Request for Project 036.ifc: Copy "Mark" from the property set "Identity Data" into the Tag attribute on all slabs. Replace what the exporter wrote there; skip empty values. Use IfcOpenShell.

First a look at what the model holds.

```python
import ifcopenshell
import ifcopenshell.util.element

model = ifcopenshell.open("Project 036.ifc")
print(model.schema)
slabs = model.by_type("IfcSlab")
print(len(slabs), "slabs")
for e in slabs[:8]:
    source = ifcopenshell.util.element.get_pset(e, "Identity Data", "Mark")
    target = e.Tag
    print(e.id(), repr(source), repr(target), sep=" | ")
```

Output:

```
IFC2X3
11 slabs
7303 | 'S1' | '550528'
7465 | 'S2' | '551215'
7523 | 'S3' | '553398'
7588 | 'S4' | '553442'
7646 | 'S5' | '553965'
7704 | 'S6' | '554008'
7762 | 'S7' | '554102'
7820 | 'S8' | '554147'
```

```python
import ifcopenshell
import ifcopenshell.util.element

model = ifcopenshell.open("Project 036.ifc")

count = 0
for e in model.by_type("IfcSlab"):
    value = ifcopenshell.util.element.get_pset(e, "Identity Data", "Mark")
    current = e.Tag
    if not value or not value.strip() or current == value:
        continue
    e.Tag = value
    count += 1

print(count, "slabs updated")

model.write("Project 036_v2.ifc")
```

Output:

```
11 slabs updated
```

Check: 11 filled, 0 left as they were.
